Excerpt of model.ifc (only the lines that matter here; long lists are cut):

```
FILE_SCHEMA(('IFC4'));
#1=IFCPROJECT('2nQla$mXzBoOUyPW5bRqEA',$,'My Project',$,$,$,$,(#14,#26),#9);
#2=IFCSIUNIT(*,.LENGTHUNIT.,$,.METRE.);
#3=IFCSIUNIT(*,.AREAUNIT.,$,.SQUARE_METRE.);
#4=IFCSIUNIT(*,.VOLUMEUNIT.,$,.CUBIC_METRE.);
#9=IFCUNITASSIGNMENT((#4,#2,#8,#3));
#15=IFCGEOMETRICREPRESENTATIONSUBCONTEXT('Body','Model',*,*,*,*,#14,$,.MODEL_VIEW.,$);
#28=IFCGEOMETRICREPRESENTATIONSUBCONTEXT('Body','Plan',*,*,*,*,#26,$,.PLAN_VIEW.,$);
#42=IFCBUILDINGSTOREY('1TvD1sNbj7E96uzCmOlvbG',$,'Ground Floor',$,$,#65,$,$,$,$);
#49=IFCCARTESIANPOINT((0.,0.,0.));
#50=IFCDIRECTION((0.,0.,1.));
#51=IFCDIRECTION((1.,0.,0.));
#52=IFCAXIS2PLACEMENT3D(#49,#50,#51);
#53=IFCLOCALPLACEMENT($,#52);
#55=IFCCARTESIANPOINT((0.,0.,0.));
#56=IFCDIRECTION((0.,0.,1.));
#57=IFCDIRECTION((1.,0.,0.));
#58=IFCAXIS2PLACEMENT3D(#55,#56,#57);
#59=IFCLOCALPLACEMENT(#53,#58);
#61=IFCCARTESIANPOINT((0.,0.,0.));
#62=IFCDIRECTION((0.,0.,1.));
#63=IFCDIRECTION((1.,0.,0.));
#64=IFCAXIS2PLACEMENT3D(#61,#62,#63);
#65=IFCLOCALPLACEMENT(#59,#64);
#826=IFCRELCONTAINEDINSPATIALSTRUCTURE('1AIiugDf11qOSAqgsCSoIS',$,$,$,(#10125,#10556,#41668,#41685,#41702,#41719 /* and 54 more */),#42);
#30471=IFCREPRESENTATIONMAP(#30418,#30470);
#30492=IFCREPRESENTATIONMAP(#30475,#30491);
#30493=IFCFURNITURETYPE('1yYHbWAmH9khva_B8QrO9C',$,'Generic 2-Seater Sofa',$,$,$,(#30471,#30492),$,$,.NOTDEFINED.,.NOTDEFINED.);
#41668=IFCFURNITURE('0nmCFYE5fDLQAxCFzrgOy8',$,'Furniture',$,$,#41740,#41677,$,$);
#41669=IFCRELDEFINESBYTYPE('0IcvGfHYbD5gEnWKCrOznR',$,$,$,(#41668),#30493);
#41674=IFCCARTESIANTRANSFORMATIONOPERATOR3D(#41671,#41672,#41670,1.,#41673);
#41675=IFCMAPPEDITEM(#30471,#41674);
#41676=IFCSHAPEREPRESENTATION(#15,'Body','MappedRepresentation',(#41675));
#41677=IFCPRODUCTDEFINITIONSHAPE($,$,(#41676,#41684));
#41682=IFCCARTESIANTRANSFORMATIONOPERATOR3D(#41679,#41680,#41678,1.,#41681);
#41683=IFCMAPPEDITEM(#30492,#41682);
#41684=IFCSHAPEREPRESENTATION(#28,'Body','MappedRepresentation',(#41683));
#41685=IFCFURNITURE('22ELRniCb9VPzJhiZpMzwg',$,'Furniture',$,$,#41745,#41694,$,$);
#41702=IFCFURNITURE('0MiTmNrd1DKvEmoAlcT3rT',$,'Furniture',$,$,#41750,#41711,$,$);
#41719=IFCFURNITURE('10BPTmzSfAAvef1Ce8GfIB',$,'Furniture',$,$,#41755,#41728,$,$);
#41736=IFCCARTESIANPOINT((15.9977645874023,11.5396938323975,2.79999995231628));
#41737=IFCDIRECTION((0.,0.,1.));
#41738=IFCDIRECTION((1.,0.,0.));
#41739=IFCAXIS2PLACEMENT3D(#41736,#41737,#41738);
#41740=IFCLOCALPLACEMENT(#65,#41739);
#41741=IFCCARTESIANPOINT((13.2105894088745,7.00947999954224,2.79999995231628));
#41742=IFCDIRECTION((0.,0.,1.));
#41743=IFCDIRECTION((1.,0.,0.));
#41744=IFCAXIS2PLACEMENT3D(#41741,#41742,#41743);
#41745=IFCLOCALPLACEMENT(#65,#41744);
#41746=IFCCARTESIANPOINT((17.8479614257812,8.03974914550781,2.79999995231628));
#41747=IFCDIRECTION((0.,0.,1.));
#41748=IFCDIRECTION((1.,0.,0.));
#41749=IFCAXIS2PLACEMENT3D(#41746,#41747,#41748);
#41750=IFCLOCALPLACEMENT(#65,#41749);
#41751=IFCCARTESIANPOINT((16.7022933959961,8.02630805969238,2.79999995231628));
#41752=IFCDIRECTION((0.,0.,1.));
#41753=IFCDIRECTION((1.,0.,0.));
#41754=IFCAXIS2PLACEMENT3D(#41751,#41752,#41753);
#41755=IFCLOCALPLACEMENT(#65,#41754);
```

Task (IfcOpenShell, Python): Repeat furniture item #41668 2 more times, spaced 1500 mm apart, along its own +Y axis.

```python
import ifcopenshell
import ifcopenshell.api.geometry
import ifcopenshell.api.root
import ifcopenshell.util.element
import ifcopenshell.util.placement
import ifcopenshell.util.unit

model = ifcopenshell.open("model.ifc")
unit_scale = ifcopenshell.util.unit.calculate_unit_scale(model)

source = model.by_id(41668)
base = ifcopenshell.util.placement.get_local_placement(source.ObjectPlacement)
step = base[:3, 1] * 1.5 / unit_scale

for i in range(1, 3):
    copy = ifcopenshell.api.root.copy_class(model, product=source)
    copy.Representation = ifcopenshell.util.element.copy_deep(
        model, source.Representation, exclude=["IfcGeometricRepresentationContext", "IfcRepresentationMap"]
    )
    matrix = base.copy()
    matrix[:3, 3] += i * step
    print("added at", matrix[:3, 3].round(3) + 0.0)
    ifcopenshell.api.geometry.edit_object_placement(model, product=copy, matrix=matrix, is_si=False)

model.write("model_rev.ifc")
```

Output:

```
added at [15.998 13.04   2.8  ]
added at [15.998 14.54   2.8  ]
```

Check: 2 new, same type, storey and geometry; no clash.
